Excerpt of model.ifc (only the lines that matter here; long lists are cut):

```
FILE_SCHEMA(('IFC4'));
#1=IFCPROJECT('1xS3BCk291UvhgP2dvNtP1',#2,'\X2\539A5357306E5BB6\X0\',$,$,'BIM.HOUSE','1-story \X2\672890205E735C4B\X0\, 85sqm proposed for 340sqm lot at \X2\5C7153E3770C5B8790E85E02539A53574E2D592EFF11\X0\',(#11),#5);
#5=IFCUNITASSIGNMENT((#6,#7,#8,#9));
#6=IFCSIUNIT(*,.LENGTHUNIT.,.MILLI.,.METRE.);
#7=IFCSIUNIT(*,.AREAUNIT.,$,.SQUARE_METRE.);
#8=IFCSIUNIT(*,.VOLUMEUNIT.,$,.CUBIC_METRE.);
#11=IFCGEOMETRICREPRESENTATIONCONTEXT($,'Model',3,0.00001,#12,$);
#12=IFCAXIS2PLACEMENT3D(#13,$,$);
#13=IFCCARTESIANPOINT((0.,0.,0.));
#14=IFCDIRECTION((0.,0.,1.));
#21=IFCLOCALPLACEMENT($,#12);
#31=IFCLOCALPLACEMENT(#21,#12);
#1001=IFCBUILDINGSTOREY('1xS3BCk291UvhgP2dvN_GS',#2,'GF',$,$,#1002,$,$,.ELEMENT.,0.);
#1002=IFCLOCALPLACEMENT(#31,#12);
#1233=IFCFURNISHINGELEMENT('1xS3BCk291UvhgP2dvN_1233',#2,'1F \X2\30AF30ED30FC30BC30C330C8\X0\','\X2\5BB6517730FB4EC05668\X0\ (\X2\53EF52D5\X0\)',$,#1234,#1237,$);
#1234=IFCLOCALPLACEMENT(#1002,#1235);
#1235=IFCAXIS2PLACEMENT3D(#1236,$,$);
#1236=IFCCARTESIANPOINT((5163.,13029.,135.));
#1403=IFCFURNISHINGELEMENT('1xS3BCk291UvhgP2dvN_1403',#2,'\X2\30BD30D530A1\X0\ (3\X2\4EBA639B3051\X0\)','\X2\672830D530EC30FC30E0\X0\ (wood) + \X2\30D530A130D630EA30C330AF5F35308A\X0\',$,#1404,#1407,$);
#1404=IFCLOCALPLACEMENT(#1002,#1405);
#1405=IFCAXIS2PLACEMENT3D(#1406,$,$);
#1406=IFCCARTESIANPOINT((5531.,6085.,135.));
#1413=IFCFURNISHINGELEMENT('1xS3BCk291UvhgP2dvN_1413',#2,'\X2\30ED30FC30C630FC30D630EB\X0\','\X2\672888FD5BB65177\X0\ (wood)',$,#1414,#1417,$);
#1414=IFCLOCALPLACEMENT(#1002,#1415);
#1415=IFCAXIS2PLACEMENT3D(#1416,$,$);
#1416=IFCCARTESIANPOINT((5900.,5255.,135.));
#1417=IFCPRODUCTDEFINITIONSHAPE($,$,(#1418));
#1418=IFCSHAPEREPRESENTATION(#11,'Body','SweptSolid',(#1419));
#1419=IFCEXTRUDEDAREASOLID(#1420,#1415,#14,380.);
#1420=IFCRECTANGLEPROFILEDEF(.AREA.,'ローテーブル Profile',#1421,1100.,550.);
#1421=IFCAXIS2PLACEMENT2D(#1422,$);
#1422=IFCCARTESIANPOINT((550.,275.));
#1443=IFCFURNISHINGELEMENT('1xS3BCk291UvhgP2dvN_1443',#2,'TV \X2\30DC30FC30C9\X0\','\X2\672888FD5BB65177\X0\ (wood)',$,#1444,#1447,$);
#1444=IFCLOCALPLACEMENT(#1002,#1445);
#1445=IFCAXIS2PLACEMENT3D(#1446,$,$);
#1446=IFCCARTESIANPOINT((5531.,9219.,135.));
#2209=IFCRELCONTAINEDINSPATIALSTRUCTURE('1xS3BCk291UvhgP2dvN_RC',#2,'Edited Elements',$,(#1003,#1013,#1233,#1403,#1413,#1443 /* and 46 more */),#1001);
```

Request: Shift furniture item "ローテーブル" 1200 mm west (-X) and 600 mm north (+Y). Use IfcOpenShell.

```python
import ifcopenshell
import ifcopenshell.api.geometry
import ifcopenshell.util.placement
import ifcopenshell.util.unit

model = ifcopenshell.open("model.ifc")
unit_scale = ifcopenshell.util.unit.calculate_unit_scale(model)

item = model.by_id(1413)
matrix = ifcopenshell.util.placement.get_local_placement(item.ObjectPlacement)
matrix[0, 3] -= 1.2 / unit_scale
matrix[1, 3] += 0.6 / unit_scale
ifcopenshell.api.geometry.edit_object_placement(model, product=item, matrix=matrix, is_si=False)

print(ifcopenshell.util.placement.get_local_placement(item.ObjectPlacement).round(3) + 0.0)

model.write("model_edited.ifc")
```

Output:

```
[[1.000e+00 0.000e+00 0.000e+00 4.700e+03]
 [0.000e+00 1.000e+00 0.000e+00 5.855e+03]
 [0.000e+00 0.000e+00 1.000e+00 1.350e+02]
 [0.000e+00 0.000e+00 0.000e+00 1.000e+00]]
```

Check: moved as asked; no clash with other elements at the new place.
